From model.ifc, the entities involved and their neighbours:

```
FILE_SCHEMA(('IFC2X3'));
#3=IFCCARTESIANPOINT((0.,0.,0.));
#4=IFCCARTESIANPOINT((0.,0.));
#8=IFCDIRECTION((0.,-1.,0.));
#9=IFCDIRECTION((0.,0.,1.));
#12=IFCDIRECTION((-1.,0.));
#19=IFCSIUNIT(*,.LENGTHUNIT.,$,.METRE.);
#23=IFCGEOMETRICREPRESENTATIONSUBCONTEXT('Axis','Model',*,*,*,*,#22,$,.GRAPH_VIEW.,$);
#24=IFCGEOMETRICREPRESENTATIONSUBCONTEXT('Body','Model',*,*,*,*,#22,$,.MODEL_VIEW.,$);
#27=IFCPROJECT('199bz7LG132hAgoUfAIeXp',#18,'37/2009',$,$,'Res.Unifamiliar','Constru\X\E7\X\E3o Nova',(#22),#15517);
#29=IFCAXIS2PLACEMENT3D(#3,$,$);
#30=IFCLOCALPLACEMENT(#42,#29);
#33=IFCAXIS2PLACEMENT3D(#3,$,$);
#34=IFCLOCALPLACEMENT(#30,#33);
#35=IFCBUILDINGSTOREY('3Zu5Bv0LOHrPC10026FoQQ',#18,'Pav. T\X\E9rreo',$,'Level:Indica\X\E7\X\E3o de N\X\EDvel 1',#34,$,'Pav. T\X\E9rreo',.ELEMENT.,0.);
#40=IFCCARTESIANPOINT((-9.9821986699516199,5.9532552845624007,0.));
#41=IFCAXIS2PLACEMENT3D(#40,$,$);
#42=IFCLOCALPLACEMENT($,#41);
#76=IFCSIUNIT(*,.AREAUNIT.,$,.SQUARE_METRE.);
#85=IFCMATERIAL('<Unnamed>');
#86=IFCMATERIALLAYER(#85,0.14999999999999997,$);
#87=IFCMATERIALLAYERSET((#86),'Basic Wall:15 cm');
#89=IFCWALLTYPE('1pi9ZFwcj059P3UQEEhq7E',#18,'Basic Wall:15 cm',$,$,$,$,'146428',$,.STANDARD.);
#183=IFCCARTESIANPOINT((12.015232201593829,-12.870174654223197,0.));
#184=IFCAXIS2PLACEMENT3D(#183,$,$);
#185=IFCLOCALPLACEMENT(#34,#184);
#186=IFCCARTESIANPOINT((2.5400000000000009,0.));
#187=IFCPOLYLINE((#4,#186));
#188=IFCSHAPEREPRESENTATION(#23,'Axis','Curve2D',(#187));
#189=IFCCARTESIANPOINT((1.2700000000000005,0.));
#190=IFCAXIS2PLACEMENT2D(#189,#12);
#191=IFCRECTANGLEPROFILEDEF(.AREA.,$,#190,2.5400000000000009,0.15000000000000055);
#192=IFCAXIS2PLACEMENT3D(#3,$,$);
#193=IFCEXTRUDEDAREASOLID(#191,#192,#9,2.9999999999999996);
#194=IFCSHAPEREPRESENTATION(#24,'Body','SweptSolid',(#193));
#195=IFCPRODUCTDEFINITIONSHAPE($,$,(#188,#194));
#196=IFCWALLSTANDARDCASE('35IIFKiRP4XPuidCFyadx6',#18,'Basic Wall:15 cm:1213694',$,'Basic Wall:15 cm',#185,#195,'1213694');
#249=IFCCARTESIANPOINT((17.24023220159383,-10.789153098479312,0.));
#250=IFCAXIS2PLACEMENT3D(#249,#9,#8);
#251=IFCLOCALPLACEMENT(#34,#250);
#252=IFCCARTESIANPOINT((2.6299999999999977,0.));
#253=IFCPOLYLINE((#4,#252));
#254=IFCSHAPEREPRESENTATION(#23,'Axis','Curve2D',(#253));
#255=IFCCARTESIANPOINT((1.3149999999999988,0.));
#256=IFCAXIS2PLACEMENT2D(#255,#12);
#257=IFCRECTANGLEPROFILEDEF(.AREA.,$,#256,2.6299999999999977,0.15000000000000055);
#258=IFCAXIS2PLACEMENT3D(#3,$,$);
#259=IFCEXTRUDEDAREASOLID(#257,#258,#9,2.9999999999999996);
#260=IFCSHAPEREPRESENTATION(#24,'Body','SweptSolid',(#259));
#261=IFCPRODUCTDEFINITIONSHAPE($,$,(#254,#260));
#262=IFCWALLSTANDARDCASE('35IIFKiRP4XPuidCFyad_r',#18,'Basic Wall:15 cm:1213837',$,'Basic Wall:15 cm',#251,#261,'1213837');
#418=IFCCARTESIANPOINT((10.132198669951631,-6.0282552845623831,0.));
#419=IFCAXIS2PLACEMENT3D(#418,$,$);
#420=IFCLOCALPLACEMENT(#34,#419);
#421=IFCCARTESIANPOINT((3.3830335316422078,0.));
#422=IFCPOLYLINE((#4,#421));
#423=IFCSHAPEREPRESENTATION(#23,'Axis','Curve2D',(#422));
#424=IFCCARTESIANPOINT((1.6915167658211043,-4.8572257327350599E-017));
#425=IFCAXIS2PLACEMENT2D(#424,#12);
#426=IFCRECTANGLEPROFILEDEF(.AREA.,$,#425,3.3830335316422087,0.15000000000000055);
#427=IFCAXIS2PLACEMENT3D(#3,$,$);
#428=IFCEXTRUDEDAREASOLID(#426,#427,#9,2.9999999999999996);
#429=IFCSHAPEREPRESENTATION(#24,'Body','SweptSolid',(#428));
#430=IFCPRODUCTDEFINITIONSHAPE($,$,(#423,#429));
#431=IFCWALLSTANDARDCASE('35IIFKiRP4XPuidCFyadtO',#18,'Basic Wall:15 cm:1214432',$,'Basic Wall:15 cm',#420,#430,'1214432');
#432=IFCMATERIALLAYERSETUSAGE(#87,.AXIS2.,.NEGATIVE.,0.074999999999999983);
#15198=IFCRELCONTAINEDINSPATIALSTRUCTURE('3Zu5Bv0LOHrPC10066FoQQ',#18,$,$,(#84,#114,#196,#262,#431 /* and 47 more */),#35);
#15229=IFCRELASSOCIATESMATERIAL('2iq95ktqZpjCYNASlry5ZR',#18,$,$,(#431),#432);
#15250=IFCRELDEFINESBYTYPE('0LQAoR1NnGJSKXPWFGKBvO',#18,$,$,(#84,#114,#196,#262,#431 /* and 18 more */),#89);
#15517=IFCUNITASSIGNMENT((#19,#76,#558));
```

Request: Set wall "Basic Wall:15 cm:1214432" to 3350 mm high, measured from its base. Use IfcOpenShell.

```python
import ifcopenshell
import ifcopenshell.geom
import ifcopenshell.util.representation
import ifcopenshell.util.shape

model = ifcopenshell.open("model.ifc")
settings = ifcopenshell.geom.settings()


def volume(element):
    """Net volume in cubic metres, openings subtracted."""
    shape = ifcopenshell.geom.create_shape(settings, element)
    return ifcopenshell.util.shape.get_volume(shape.geometry)


wall = model.by_guid("35IIFKiRP4XPuidCFyadtO")
before = volume(wall)

body = ifcopenshell.util.representation.get_representation(wall, "Model", "Body")
solid = body.Items[0]
old_height = solid.Depth
solid.Depth = 3.35
after = volume(wall)

print(f"height {old_height:g} -> {solid.Depth:g}, volume {before:.3f} -> {after:.3f} m3")

model.write("model_v2.ifc")
```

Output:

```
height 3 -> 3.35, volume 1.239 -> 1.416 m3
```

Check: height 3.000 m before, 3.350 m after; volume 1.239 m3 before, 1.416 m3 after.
